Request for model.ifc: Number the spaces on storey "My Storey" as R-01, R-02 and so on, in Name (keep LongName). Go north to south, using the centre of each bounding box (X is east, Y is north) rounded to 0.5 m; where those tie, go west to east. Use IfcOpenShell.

First a look at what the model holds.

```python
import ifcopenshell
import ifcopenshell.util.element
import ifcopenshell.util.placement

model = ifcopenshell.open("model.ifc")
print(model.schema)
storey = next(s for s in model.by_type("IfcBuildingStorey") if s.Name == "My Storey")
spaces = [e for e in ifcopenshell.util.element.get_decomposition(storey) if e.is_a("IfcSpace")]
for e in sorted(spaces, key=lambda e: e.id()):
    origin = ifcopenshell.util.placement.get_local_placement(e.ObjectPlacement)[:3, 3]
    print(e.id(), e.Name, e.LongName, origin.round(2) + 0.0, sep=" | ")
```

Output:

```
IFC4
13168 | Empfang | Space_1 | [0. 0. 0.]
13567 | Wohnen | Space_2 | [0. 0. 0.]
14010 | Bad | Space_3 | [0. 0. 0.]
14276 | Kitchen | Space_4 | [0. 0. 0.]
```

```python
import ifcopenshell
import ifcopenshell.geom
import ifcopenshell.util.element
import ifcopenshell.util.shape

model = ifcopenshell.open("model.ifc")
settings = ifcopenshell.geom.settings()
settings.set("use-world-coords", True)


def centre(element):
    shape = ifcopenshell.geom.create_shape(settings, element)
    return ifcopenshell.util.shape.get_bbox_centroid(shape.geometry)


storey = next(s for s in model.by_type("IfcBuildingStorey") if s.Name == "My Storey")
spaces = [e for e in ifcopenshell.util.element.get_decomposition(storey) if e.is_a("IfcSpace")]

# Insertion points can sit at a corner or the storey origin, so sort by the geometry (in metres).
centres = {e: centre(e) for e in spaces}
spaces.sort(key=lambda e: (-round(centres[e][1] / 0.5), centres[e][0]))

for i, e in enumerate(spaces, start=1):
    number = f"R-{i:02d}"
    e.Name = number
    print(e.id(), number)

model.write("model_edited.ifc")
```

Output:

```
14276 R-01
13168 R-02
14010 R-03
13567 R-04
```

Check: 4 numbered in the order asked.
